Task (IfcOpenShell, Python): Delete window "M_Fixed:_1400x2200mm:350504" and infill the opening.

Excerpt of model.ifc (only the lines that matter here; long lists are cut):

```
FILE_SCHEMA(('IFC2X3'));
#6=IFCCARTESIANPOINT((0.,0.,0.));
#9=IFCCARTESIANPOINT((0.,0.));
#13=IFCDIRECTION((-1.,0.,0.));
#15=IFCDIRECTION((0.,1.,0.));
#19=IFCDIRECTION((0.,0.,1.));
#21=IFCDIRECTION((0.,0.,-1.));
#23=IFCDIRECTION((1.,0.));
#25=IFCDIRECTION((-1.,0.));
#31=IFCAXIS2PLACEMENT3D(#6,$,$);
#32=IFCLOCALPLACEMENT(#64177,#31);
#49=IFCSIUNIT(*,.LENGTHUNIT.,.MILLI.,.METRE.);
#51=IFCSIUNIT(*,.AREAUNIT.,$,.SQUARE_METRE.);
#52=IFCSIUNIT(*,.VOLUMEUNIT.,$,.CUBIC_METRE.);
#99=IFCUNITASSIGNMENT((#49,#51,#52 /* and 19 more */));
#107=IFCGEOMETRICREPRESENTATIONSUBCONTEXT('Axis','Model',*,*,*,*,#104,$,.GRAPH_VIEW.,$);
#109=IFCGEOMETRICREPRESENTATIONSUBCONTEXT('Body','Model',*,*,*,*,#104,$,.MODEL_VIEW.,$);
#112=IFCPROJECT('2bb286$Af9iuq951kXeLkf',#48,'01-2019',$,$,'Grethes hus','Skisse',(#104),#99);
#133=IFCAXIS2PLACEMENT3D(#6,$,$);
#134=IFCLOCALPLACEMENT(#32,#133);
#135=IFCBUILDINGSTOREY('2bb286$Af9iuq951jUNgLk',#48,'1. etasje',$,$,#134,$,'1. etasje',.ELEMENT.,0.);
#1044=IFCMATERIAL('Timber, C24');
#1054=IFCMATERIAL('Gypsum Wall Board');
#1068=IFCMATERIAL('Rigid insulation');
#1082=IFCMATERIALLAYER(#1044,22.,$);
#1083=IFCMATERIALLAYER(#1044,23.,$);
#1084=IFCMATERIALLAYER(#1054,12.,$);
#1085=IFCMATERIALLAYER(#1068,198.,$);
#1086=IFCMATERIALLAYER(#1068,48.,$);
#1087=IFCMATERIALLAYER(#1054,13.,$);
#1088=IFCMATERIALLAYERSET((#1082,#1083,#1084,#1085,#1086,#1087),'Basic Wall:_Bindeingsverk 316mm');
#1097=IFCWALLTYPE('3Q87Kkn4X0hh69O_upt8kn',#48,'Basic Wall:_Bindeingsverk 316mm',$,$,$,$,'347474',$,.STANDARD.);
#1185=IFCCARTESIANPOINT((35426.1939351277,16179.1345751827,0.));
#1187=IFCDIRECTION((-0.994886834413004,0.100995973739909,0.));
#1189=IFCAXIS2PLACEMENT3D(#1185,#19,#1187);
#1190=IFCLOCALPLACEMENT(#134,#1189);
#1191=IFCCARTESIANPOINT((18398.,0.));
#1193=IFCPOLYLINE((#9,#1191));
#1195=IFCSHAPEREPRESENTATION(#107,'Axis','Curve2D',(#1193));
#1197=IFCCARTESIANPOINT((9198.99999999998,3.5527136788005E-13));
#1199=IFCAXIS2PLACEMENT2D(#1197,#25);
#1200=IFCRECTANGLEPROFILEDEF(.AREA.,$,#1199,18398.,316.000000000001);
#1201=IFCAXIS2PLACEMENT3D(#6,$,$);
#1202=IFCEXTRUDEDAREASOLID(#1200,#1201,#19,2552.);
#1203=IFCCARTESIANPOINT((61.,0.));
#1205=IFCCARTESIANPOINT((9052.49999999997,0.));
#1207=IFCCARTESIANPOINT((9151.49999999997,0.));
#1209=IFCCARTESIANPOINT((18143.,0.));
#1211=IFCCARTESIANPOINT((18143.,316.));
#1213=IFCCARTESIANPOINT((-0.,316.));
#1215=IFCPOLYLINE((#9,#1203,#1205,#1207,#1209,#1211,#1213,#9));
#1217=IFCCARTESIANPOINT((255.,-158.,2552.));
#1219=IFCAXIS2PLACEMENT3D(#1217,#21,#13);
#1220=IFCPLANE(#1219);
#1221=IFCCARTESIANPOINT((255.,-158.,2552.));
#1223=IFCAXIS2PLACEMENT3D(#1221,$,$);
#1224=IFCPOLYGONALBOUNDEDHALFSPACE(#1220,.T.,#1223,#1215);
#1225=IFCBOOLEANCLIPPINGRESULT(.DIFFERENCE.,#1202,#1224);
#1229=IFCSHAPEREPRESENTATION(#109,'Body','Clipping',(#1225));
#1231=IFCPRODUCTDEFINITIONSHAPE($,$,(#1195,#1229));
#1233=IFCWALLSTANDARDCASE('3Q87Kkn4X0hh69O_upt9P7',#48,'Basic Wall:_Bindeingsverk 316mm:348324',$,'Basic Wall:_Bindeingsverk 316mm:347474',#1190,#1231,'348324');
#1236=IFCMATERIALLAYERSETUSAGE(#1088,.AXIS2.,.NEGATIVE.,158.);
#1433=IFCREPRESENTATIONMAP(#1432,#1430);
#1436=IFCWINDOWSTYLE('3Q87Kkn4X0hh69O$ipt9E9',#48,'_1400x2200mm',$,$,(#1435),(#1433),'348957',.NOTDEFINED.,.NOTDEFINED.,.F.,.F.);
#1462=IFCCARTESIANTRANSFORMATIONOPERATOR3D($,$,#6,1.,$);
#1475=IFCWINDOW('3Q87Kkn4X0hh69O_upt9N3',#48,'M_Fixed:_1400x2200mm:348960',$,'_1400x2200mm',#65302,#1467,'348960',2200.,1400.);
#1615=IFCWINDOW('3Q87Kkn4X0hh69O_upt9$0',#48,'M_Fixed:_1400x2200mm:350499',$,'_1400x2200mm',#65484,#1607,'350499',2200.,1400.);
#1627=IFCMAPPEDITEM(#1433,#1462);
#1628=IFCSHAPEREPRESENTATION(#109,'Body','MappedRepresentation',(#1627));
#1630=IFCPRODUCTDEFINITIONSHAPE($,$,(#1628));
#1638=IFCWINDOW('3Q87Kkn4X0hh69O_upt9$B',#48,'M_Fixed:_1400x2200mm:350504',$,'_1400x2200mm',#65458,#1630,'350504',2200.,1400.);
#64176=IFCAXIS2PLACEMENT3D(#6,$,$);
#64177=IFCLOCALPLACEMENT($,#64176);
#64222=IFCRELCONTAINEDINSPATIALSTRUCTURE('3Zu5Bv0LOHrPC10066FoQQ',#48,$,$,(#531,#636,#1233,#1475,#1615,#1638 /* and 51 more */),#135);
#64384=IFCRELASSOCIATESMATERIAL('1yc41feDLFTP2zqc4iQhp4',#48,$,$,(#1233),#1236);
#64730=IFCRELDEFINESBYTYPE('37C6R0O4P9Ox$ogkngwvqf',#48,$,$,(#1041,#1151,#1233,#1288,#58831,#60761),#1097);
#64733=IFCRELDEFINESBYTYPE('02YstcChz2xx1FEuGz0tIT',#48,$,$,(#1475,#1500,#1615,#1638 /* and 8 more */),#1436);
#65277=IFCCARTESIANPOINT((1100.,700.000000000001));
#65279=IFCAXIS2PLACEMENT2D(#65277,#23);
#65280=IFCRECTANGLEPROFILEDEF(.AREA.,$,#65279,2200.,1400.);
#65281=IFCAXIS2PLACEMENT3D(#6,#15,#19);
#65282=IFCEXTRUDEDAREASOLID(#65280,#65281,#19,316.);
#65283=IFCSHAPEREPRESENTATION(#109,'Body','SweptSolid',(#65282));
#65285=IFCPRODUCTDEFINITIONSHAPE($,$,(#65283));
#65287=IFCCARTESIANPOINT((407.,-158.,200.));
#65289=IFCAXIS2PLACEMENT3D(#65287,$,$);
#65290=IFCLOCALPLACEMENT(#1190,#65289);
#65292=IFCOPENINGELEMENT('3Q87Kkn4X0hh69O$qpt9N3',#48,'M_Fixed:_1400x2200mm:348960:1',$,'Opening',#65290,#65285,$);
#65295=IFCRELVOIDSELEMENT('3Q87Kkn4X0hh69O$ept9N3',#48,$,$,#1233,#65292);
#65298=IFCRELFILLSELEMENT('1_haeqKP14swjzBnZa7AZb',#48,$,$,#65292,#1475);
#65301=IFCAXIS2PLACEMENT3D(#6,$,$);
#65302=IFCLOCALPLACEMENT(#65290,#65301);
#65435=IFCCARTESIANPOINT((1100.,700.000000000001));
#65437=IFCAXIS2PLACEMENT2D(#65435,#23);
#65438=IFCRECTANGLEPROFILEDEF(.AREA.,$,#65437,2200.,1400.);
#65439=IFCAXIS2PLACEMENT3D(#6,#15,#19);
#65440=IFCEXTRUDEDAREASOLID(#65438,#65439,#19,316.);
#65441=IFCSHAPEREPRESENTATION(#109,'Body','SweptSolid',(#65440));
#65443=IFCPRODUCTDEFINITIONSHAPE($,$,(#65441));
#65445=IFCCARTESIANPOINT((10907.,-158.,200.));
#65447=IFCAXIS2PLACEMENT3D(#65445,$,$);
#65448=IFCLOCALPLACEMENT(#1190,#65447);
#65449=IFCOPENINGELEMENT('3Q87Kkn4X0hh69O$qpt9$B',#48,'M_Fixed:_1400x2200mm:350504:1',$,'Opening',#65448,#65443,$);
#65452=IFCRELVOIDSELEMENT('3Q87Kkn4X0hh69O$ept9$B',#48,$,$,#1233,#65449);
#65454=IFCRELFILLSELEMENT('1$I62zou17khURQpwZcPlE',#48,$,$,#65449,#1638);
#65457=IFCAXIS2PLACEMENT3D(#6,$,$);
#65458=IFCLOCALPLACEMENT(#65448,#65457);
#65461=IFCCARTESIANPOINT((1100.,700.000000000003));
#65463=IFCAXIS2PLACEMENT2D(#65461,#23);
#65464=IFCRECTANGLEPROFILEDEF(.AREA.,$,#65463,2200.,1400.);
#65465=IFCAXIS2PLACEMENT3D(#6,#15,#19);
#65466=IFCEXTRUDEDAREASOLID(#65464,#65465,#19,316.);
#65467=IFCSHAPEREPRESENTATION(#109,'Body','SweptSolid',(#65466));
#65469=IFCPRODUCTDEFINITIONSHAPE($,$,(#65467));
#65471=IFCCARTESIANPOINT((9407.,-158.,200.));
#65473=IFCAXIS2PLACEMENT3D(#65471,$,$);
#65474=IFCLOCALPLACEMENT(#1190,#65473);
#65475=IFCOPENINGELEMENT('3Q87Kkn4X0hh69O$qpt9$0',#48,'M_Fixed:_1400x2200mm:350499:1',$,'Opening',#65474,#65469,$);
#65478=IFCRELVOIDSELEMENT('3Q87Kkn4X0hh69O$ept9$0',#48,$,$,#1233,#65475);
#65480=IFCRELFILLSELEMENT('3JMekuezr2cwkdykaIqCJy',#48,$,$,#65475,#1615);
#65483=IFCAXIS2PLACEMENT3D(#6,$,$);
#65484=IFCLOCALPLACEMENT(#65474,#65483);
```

```python
import ifcopenshell
import ifcopenshell.api.feature
import ifcopenshell.api.root
import ifcopenshell.geom
import ifcopenshell.util.shape

model = ifcopenshell.open("model.ifc")
settings = ifcopenshell.geom.settings()


def volume(element):
    """Net volume in cubic metres, openings subtracted."""
    shape = ifcopenshell.geom.create_shape(settings, element)
    return ifcopenshell.util.shape.get_volume(shape.geometry)


window = model.by_guid("3Q87Kkn4X0hh69O_upt9$B")
opening = window.FillsVoids[0].RelatingOpeningElement
wall = opening.VoidsElements[0].RelatingBuildingElement
before = volume(wall)

ifcopenshell.api.root.remove_product(model, product=window)
ifcopenshell.api.feature.remove_feature(model, feature=opening)

after = volume(wall)

print(f"wall volume {before:.3f} -> {after:.3f} m3")

model.write("model_updated.ifc")
```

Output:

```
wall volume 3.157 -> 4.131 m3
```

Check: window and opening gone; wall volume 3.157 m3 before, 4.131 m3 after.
